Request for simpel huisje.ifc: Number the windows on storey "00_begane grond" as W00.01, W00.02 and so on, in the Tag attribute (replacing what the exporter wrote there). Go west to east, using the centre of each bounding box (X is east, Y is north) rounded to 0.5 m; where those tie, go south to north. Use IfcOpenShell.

First a look at what the model holds.

```python
import ifcopenshell
import ifcopenshell.util.element
import ifcopenshell.util.placement

model = ifcopenshell.open("simpel huisje.ifc")
print(model.schema)
storey = next(s for s in model.by_type("IfcBuildingStorey") if s.Name == "00_begane grond")
windows = [e for e in ifcopenshell.util.element.get_decomposition(storey) if e.is_a("IfcWindow")]
for e in sorted(windows, key=lambda e: e.id()):
    origin = ifcopenshell.util.placement.get_local_placement(e.ObjectPlacement)[:3, 3]
    print(e.id(), e.Tag, e.Name, origin.round(2) + 0.0, sep=" | ")
```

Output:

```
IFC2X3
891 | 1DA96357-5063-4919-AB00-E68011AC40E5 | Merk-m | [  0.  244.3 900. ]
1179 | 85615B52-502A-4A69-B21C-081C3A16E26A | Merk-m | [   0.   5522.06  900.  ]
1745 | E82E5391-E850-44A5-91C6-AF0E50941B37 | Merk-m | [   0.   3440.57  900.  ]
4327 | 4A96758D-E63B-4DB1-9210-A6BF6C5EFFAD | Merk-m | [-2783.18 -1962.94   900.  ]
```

```python
import ifcopenshell
import ifcopenshell.geom
import ifcopenshell.util.element
import ifcopenshell.util.shape

model = ifcopenshell.open("simpel huisje.ifc")
settings = ifcopenshell.geom.settings()
settings.set("use-world-coords", True)


def centre(element):
    shape = ifcopenshell.geom.create_shape(settings, element)
    return ifcopenshell.util.shape.get_bbox_centroid(shape.geometry)


storey = next(s for s in model.by_type("IfcBuildingStorey") if s.Name == "00_begane grond")
windows = [e for e in ifcopenshell.util.element.get_decomposition(storey) if e.is_a("IfcWindow")]

# Insertion points can sit at a corner or the storey origin, so sort by the geometry (in metres).
centres = {e: centre(e) for e in windows}
windows.sort(key=lambda e: (round(centres[e][0] / 0.5), centres[e][1]))

for i, e in enumerate(windows, start=1):
    number = f"W00.{i:02d}"
    e.Tag = number
    print(e.id(), number)

model.write("simpel huisje_updated.ifc")
```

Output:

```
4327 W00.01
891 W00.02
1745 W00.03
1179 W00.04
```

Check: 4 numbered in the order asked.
